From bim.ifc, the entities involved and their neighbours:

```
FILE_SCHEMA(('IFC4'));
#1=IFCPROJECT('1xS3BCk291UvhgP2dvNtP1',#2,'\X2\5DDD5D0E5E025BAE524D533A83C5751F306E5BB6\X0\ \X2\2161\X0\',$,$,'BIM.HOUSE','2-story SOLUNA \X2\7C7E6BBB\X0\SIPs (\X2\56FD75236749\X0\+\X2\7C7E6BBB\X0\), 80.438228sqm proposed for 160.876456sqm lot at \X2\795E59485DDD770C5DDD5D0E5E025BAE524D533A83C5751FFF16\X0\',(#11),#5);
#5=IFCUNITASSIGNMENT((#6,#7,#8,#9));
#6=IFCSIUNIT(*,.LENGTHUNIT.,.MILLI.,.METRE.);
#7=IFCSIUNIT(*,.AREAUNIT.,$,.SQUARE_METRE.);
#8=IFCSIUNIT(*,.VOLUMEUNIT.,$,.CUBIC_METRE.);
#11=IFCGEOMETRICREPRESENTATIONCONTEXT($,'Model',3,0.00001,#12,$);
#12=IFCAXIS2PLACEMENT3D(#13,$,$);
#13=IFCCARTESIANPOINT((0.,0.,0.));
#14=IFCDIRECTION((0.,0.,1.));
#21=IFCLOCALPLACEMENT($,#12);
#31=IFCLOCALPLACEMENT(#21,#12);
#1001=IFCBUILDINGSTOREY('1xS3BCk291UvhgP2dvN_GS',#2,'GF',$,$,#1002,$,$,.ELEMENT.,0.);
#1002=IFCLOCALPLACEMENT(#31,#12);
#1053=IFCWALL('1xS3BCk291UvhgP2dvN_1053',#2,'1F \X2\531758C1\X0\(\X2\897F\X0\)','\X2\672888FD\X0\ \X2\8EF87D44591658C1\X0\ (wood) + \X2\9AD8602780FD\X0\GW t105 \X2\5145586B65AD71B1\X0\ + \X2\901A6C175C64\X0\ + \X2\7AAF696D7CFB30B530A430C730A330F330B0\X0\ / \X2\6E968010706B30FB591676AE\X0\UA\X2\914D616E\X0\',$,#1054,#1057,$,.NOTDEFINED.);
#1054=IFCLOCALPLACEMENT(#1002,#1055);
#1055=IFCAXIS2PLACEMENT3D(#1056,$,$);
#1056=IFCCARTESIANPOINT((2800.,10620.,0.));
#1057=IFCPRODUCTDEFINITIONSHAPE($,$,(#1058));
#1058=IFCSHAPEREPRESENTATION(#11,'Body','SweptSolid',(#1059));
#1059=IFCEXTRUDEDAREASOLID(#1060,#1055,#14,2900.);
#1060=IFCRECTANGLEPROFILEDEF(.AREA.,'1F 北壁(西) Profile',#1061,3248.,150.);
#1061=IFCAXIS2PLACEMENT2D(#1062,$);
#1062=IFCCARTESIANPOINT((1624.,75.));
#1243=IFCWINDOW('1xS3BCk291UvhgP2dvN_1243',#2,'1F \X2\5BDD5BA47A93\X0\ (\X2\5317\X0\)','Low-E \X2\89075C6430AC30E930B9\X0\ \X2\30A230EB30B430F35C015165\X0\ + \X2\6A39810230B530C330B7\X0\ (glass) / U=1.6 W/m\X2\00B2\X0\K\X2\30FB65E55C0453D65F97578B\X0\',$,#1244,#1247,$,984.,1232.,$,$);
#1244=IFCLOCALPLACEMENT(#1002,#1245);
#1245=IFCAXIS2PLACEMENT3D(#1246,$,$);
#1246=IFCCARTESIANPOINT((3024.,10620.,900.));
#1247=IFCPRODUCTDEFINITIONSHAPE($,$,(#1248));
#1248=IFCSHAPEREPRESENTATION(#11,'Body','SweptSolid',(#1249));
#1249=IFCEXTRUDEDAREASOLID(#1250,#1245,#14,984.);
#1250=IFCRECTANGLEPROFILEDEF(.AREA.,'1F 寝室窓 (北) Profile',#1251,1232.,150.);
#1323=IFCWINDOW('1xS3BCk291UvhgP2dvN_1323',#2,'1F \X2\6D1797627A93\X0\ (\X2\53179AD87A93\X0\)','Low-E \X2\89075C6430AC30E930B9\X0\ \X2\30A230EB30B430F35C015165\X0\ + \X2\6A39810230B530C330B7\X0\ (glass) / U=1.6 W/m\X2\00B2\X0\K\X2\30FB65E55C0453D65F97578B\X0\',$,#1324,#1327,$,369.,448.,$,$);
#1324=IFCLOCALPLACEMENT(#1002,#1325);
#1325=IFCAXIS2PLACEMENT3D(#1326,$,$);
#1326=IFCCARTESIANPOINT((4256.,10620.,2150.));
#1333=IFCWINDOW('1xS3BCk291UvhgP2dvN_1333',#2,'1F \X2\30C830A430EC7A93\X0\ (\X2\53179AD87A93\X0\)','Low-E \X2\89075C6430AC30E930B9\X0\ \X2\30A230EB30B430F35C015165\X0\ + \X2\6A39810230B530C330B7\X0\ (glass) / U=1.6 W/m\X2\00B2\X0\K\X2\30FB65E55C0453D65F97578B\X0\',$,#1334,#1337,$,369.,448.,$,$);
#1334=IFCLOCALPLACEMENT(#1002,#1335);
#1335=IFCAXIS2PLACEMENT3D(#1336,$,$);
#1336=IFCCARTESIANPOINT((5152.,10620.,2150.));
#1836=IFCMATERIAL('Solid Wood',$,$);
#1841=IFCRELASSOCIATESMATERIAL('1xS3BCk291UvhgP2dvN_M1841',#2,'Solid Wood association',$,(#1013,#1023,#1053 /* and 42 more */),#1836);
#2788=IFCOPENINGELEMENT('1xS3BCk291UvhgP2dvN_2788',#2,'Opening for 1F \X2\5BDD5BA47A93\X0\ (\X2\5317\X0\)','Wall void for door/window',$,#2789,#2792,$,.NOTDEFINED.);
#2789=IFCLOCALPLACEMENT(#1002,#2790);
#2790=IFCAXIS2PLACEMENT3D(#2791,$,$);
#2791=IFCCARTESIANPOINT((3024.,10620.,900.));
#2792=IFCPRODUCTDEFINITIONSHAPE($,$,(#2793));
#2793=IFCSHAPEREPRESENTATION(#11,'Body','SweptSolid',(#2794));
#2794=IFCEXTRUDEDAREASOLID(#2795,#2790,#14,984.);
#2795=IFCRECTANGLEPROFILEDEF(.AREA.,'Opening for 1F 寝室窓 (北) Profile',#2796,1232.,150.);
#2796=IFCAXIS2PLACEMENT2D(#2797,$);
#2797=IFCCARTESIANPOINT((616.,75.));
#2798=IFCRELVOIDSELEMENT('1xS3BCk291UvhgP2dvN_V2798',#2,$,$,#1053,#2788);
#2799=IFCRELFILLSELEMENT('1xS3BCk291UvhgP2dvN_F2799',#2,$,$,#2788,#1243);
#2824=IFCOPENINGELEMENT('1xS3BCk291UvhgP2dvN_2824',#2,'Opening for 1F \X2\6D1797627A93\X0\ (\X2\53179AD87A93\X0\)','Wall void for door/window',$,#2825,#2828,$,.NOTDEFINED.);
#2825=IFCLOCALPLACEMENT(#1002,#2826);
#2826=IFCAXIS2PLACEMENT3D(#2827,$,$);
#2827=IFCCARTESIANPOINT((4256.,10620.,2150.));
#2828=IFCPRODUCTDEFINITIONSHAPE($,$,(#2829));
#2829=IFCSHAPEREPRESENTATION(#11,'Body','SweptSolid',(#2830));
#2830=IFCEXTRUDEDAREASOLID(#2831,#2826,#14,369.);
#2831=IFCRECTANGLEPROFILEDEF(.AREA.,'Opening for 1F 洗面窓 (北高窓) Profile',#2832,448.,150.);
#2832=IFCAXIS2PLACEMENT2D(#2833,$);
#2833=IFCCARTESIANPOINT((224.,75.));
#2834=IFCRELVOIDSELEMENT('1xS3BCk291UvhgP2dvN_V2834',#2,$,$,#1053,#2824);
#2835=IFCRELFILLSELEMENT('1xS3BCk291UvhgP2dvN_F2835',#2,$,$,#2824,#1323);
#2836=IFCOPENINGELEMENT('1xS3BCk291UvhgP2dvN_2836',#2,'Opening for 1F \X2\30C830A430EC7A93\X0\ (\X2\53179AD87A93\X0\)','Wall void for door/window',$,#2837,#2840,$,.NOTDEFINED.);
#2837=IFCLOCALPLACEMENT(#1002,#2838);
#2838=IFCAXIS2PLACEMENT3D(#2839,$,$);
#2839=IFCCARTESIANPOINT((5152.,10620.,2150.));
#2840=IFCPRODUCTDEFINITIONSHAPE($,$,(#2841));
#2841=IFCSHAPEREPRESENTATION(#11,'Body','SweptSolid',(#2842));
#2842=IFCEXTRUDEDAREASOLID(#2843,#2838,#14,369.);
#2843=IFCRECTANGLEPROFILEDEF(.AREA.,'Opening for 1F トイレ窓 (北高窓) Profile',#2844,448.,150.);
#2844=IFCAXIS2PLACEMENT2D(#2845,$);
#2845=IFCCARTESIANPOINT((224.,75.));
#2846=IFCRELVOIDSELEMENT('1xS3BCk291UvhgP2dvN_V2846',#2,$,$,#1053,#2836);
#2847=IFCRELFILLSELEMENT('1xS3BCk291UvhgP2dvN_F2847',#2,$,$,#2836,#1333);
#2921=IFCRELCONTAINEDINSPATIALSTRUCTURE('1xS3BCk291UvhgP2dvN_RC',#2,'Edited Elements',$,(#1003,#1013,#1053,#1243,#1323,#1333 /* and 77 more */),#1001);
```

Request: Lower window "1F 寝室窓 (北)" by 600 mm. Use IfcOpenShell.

```python
import numpy as np
import ifcopenshell
import ifcopenshell.api.geometry
import ifcopenshell.util.placement
import ifcopenshell.util.unit

model = ifcopenshell.open("bim.ifc")
unit_scale = ifcopenshell.util.unit.calculate_unit_scale(model)

window = model.by_guid("1xS3BCk291UvhgP2dvN_1243")
opening = window.FillsVoids[0].RelatingOpeningElement
dz = -0.6 / unit_scale

shift = np.array([0.0, 0.0, dz])
# The window is not placed relative to its opening, so move both.
for product in (opening, window):
    matrix = ifcopenshell.util.placement.get_local_placement(product.ObjectPlacement)
    matrix[:3, 3] += shift
    ifcopenshell.api.geometry.edit_object_placement(model, product=product, matrix=matrix, is_si=False)

print(f"moved by {dz * unit_scale:+.3f} m")

model.write("bim_updated.ifc")
```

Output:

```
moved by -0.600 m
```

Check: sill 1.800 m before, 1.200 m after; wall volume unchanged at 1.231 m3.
